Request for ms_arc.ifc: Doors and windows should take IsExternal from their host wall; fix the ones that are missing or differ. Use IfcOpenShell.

First a look at what the model holds.

```python
import ifcopenshell
import ifcopenshell.util.element

model = ifcopenshell.open("ms_arc.ifc")
print(model.schema)
seen = {}
for e in model.by_type("IfcDoor") + model.by_type("IfcWindow"):
    if not e.FillsVoids:
        continue
    host = e.FillsVoids[0].RelatingOpeningElement.VoidsElements[0].RelatingBuildingElement
    own = ifcopenshell.util.element.get_pset(e, f"Pset_{e.is_a()[3:].removesuffix('StandardCase')}Common", "IsExternal")
    wall = ifcopenshell.util.element.get_pset(host, "Pset_WallCommon", "IsExternal")
    seen[e.is_a(), own, wall] = seen.get((e.is_a(), own, wall), 0) + 1
for (cls, own, wall), count in sorted(seen.items(), key=str):
    print(count, cls, "IsExternal:", own, "| host wall:", wall)
```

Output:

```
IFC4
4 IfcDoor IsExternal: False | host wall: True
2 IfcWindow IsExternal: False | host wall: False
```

```python
import ifcopenshell
import ifcopenshell.api.pset
import ifcopenshell.util.element

model = ifcopenshell.open("ms_arc.ifc")

count = 0
for ifc_class, pset_name in (("IfcDoor", "Pset_DoorCommon"), ("IfcWindow", "Pset_WindowCommon")):
    for e in model.by_type(ifc_class):
        if not e.FillsVoids:
            continue
        host = e.FillsVoids[0].RelatingOpeningElement.VoidsElements[0].RelatingBuildingElement
        external = ifcopenshell.util.element.get_pset(host, "Pset_WallCommon", "IsExternal")
        if external is None or ifcopenshell.util.element.get_pset(e, pset_name, "IsExternal") == external:
            continue
        pset = ifcopenshell.api.pset.add_pset(model, product=e, name=pset_name)
        ifcopenshell.api.pset.edit_pset(model, pset=pset, properties={"IsExternal": external})
        count += 1

print(count, "updated")

model.write("ms_arc_updated.ifc")
```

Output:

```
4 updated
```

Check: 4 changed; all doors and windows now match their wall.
